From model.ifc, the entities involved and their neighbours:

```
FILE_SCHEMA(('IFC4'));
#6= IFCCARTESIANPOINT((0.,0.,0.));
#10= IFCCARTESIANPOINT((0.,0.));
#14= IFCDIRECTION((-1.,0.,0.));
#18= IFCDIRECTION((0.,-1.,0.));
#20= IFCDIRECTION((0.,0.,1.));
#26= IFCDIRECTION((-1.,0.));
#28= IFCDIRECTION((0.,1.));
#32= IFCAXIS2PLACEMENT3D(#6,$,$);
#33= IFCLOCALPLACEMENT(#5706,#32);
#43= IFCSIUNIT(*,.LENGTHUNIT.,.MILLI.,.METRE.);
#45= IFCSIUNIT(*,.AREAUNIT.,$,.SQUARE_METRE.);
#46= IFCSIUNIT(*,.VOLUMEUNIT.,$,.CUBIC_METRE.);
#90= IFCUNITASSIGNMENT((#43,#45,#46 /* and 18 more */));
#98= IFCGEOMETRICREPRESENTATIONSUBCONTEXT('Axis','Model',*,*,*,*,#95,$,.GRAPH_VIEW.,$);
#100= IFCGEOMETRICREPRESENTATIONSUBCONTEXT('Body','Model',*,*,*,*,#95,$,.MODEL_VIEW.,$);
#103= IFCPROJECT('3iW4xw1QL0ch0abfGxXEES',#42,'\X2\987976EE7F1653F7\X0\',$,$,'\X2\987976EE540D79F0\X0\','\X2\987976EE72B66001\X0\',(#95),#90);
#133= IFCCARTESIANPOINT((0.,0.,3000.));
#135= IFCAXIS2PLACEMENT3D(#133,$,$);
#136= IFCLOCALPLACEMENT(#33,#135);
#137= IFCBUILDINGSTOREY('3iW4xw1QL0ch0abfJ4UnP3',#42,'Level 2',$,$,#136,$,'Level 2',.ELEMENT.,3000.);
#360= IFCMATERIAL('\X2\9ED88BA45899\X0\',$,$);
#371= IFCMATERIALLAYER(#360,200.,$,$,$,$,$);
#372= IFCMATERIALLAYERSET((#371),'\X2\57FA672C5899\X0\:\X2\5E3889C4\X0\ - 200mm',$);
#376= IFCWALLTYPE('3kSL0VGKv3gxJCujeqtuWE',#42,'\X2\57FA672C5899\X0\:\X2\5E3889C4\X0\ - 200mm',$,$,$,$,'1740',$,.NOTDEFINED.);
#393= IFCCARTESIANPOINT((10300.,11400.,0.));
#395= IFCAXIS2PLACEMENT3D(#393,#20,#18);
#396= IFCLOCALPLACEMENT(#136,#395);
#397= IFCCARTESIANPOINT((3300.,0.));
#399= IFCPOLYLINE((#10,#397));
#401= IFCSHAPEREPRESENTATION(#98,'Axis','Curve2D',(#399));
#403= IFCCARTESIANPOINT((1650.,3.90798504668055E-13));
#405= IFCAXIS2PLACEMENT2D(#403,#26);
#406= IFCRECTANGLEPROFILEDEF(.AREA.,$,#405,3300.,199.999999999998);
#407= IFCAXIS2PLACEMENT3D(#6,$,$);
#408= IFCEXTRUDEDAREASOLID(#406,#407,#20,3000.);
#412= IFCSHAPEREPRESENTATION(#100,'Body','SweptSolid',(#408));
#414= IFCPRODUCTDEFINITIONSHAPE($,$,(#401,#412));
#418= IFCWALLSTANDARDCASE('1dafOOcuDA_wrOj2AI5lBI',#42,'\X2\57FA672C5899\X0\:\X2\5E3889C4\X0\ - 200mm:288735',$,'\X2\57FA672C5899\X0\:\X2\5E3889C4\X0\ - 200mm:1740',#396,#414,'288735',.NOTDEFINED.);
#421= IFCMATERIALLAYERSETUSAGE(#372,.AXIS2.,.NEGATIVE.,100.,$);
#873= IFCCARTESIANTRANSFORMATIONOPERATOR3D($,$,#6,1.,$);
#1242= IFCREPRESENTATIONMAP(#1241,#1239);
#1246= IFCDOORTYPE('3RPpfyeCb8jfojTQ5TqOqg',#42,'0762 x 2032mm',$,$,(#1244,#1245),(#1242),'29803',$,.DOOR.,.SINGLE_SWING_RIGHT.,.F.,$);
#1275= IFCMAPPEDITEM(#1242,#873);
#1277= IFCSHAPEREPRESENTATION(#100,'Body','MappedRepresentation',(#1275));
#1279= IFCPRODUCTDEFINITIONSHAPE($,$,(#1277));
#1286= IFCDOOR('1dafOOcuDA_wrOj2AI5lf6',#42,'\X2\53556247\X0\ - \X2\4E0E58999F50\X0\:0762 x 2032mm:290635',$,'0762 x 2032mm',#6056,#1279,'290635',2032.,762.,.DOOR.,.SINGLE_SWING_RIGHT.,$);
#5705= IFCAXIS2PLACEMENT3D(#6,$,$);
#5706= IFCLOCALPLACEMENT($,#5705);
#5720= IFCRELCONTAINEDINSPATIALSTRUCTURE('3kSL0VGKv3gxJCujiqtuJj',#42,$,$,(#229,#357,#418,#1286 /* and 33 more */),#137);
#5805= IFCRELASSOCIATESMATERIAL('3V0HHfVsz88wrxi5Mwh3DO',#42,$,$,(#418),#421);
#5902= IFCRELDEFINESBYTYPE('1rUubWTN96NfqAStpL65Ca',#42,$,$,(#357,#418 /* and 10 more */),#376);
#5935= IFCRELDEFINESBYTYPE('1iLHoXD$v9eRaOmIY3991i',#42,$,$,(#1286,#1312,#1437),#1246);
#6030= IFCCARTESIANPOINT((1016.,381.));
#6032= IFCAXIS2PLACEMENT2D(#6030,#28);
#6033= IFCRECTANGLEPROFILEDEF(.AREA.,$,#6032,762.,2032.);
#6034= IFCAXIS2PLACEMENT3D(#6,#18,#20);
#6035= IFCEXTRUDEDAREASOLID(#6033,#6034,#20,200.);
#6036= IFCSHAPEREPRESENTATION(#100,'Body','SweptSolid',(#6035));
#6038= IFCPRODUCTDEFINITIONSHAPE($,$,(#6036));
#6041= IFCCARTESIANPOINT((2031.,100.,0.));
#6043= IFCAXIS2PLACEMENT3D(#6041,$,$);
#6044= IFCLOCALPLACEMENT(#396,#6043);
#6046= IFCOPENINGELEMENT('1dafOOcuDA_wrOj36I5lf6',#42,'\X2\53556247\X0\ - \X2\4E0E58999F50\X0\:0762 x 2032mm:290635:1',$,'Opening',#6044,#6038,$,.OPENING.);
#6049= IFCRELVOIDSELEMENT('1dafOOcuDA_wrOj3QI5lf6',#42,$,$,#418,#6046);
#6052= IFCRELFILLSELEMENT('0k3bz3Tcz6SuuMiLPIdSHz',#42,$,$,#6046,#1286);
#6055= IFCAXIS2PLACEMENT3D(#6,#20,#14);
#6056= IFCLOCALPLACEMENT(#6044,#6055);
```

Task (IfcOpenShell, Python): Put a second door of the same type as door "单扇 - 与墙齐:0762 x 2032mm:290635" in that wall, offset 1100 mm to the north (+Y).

```python
import ifcopenshell
import ifcopenshell.api.feature
import ifcopenshell.api.geometry
import ifcopenshell.api.root
import ifcopenshell.geom
import ifcopenshell.util.element
import ifcopenshell.util.placement
import ifcopenshell.util.shape
import ifcopenshell.util.unit

model = ifcopenshell.open("model.ifc")
unit_scale = ifcopenshell.util.unit.calculate_unit_scale(model)
settings = ifcopenshell.geom.settings()


def volume(element):
    """Net volume in cubic metres, openings subtracted."""
    shape = ifcopenshell.geom.create_shape(settings, element)
    return ifcopenshell.util.shape.get_volume(shape.geometry)


def reuse_history(source, copy):
    """copy_class also copies each property set's owner history, people and application; keep the originals."""
    for rel in copy.IsDefinedBy:
        if rel.is_a("IfcRelDefinesByProperties") and (history := rel.RelatingPropertyDefinition.OwnerHistory):
            rel.RelatingPropertyDefinition.OwnerHistory = source.OwnerHistory
            ifcopenshell.util.element.remove_deep2(model, history)


door = model.by_id(1286)
opening = door.FillsVoids[0].RelatingOpeningElement
wall = opening.VoidsElements[0].RelatingBuildingElement
before = volume(wall)
shift = ifcopenshell.util.placement.get_local_placement(wall.ObjectPlacement)[:3, 0] * -1.1 / unit_scale

# copy_class copies the void relationship, type, container and properties, but no geometry.
new_opening = ifcopenshell.api.root.copy_class(model, product=opening)
new_opening.Representation = ifcopenshell.util.element.copy_deep(
    model, opening.Representation, exclude=["IfcGeometricRepresentationContext", "IfcRepresentationMap"]
)
new_opening.Name = "单扇 - 与墙齐:0762 x 2032mm"
new_door = ifcopenshell.api.root.copy_class(model, product=door)
new_door.Representation = ifcopenshell.util.element.copy_deep(
    model, door.Representation, exclude=["IfcGeometricRepresentationContext", "IfcRepresentationMap"]
)
new_door.Name = "单扇 - 与墙齐:0762 x 2032mm"
new_door.Tag = None
reuse_history(door, new_door)
ifcopenshell.api.feature.add_filling(model, opening=new_opening, element=new_door)

for old, new in ((opening, new_opening), (door, new_door)):
    matrix = ifcopenshell.util.placement.get_local_placement(old.ObjectPlacement)
    matrix[:3, 3] += shift
    ifcopenshell.api.geometry.edit_object_placement(model, product=new, matrix=matrix, is_si=False)

after = volume(wall)

print(f"wall volume {before:.3f} -> {after:.3f} m3")

model.write("model_rev.ifc")
```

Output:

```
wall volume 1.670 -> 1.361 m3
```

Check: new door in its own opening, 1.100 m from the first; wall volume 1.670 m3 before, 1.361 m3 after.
